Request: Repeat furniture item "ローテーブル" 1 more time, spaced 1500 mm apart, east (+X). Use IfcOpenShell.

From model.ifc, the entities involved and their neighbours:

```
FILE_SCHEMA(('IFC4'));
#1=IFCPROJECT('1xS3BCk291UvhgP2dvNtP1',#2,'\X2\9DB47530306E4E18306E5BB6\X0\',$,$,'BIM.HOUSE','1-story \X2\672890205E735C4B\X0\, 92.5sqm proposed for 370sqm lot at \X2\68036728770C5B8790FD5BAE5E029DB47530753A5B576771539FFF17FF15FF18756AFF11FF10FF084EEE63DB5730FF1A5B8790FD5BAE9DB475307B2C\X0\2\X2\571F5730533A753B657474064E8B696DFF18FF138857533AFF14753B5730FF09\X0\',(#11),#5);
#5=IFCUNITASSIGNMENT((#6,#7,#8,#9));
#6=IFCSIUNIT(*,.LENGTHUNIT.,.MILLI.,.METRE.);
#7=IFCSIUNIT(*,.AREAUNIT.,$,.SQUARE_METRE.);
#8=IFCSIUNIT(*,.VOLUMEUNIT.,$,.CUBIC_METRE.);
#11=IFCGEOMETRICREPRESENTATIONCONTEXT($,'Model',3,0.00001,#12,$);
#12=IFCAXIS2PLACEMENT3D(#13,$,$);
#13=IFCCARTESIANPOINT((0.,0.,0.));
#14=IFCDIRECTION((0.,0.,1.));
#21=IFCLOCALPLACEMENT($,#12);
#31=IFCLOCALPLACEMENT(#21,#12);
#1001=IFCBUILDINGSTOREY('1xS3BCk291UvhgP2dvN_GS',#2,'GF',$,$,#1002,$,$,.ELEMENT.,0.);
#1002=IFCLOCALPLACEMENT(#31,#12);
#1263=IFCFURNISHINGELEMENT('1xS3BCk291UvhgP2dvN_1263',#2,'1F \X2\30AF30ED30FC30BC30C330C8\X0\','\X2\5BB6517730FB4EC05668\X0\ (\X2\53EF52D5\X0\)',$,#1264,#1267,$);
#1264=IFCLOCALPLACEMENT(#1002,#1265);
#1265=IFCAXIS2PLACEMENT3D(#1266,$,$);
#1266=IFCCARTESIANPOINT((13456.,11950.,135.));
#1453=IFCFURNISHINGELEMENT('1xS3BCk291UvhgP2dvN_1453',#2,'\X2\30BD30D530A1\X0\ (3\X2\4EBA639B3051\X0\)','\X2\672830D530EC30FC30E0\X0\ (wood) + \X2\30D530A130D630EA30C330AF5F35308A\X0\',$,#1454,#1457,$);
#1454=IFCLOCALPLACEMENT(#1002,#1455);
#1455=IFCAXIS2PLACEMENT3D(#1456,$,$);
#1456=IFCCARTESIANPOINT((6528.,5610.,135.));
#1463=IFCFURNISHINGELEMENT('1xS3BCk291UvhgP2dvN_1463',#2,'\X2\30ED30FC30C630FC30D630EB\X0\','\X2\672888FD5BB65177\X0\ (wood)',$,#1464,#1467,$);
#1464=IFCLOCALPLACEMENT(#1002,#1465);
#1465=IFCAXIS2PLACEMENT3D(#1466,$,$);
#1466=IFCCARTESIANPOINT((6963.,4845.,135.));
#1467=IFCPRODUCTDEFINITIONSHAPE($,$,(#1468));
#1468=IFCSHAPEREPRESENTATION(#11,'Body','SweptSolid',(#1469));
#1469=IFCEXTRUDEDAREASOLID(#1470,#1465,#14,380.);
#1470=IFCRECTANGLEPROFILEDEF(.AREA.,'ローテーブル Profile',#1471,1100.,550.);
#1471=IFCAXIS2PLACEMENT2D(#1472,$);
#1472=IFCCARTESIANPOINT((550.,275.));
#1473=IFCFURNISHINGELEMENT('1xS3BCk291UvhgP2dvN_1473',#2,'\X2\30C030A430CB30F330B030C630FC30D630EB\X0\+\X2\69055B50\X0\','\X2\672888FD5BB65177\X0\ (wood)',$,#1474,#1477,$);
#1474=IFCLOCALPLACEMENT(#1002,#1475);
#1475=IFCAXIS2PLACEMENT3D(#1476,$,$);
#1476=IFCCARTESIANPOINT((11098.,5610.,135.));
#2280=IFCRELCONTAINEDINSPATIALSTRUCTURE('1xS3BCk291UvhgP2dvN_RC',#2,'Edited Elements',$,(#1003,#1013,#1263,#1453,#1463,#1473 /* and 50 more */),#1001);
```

```python
import numpy as np
import ifcopenshell
import ifcopenshell.api.geometry
import ifcopenshell.api.root
import ifcopenshell.util.element
import ifcopenshell.util.placement
import ifcopenshell.util.unit

model = ifcopenshell.open("model.ifc")
unit_scale = ifcopenshell.util.unit.calculate_unit_scale(model)


def reuse_history(source, copy):
    """copy_class also copies each property set's owner history, people and application; keep the originals."""
    for rel in copy.IsDefinedBy:
        if rel.is_a("IfcRelDefinesByProperties") and (history := rel.RelatingPropertyDefinition.OwnerHistory):
            rel.RelatingPropertyDefinition.OwnerHistory = source.OwnerHistory
            ifcopenshell.util.element.remove_deep2(model, history)


source = model.by_id(1463)
base = ifcopenshell.util.placement.get_local_placement(source.ObjectPlacement)
step = np.array([1.0, 0.0, 0.0]) * 1.5 / unit_scale

for i in range(1, 2):
    copy = ifcopenshell.api.root.copy_class(model, product=source)
    copy.Representation = ifcopenshell.util.element.copy_deep(
        model, source.Representation, exclude=["IfcGeometricRepresentationContext", "IfcRepresentationMap"]
    )
    reuse_history(source, copy)
    matrix = base.copy()
    matrix[:3, 3] += i * step
    print("added at", matrix[:3, 3].round(3) + 0.0)
    ifcopenshell.api.geometry.edit_object_placement(model, product=copy, matrix=matrix, is_si=False)

model.write("model_edited.ifc")
```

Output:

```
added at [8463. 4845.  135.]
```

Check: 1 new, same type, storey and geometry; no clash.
